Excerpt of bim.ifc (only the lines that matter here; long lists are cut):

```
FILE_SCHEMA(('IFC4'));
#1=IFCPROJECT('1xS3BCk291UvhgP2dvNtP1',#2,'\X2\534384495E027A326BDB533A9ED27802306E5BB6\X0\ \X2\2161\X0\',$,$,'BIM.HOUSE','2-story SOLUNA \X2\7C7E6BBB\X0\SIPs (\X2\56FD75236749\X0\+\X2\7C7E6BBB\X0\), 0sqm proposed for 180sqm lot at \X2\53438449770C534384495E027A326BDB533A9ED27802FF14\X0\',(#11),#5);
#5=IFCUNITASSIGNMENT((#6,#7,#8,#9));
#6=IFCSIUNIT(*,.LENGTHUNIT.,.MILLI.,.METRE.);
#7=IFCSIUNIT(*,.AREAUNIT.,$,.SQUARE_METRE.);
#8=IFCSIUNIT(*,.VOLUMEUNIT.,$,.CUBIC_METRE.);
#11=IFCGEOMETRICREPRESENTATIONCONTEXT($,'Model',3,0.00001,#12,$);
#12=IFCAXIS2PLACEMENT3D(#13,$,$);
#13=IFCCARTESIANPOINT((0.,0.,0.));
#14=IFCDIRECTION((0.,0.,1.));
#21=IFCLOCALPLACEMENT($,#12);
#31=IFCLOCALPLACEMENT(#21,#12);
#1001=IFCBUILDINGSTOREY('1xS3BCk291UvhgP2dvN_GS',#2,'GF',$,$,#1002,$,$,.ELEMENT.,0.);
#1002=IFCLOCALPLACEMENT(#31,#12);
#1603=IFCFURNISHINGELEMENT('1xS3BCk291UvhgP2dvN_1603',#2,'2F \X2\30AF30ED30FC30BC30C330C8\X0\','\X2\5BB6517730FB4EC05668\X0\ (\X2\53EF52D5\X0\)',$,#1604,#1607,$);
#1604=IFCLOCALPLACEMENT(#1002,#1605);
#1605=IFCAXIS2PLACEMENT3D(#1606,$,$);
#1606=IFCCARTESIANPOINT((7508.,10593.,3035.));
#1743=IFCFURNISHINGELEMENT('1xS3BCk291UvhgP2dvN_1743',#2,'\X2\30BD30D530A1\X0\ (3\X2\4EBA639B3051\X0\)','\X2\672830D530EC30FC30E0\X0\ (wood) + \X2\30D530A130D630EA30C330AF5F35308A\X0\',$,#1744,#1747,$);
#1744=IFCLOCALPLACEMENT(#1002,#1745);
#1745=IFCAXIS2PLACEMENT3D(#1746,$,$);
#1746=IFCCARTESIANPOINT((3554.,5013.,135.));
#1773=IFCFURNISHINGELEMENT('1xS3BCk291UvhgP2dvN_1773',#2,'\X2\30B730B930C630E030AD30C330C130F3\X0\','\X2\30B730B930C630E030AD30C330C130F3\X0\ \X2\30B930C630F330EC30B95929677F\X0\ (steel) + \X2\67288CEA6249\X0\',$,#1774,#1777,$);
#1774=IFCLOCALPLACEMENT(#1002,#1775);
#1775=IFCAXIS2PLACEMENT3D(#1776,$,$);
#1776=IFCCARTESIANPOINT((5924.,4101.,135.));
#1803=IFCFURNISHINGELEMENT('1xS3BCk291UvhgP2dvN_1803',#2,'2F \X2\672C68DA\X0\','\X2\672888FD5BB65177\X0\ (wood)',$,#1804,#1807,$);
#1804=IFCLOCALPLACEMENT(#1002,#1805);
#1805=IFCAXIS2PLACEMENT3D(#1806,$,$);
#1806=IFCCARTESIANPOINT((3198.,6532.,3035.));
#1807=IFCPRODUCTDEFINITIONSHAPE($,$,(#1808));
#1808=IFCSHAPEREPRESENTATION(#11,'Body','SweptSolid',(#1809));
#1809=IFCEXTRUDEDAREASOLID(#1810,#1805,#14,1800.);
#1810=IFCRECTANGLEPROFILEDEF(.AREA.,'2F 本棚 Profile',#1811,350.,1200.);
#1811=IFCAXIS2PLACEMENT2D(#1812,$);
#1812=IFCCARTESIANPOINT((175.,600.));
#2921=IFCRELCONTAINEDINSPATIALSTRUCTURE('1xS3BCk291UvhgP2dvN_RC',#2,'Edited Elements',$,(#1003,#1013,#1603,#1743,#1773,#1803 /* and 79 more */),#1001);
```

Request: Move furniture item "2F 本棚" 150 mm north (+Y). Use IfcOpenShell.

```python
import ifcopenshell
import ifcopenshell.api.geometry
import ifcopenshell.util.placement
import ifcopenshell.util.unit

model = ifcopenshell.open("bim.ifc")
unit_scale = ifcopenshell.util.unit.calculate_unit_scale(model)

item = model.by_id(1803)
matrix = ifcopenshell.util.placement.get_local_placement(item.ObjectPlacement)
matrix[1, 3] += 0.15 / unit_scale
ifcopenshell.api.geometry.edit_object_placement(model, product=item, matrix=matrix, is_si=False)

print(ifcopenshell.util.placement.get_local_placement(item.ObjectPlacement).round(3) + 0.0)

model.write("bim_edited.ifc")
```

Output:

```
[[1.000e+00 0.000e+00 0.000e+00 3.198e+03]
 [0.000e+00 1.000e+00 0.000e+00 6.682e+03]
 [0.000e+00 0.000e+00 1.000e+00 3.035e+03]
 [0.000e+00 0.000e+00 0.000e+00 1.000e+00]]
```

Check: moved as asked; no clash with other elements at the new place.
